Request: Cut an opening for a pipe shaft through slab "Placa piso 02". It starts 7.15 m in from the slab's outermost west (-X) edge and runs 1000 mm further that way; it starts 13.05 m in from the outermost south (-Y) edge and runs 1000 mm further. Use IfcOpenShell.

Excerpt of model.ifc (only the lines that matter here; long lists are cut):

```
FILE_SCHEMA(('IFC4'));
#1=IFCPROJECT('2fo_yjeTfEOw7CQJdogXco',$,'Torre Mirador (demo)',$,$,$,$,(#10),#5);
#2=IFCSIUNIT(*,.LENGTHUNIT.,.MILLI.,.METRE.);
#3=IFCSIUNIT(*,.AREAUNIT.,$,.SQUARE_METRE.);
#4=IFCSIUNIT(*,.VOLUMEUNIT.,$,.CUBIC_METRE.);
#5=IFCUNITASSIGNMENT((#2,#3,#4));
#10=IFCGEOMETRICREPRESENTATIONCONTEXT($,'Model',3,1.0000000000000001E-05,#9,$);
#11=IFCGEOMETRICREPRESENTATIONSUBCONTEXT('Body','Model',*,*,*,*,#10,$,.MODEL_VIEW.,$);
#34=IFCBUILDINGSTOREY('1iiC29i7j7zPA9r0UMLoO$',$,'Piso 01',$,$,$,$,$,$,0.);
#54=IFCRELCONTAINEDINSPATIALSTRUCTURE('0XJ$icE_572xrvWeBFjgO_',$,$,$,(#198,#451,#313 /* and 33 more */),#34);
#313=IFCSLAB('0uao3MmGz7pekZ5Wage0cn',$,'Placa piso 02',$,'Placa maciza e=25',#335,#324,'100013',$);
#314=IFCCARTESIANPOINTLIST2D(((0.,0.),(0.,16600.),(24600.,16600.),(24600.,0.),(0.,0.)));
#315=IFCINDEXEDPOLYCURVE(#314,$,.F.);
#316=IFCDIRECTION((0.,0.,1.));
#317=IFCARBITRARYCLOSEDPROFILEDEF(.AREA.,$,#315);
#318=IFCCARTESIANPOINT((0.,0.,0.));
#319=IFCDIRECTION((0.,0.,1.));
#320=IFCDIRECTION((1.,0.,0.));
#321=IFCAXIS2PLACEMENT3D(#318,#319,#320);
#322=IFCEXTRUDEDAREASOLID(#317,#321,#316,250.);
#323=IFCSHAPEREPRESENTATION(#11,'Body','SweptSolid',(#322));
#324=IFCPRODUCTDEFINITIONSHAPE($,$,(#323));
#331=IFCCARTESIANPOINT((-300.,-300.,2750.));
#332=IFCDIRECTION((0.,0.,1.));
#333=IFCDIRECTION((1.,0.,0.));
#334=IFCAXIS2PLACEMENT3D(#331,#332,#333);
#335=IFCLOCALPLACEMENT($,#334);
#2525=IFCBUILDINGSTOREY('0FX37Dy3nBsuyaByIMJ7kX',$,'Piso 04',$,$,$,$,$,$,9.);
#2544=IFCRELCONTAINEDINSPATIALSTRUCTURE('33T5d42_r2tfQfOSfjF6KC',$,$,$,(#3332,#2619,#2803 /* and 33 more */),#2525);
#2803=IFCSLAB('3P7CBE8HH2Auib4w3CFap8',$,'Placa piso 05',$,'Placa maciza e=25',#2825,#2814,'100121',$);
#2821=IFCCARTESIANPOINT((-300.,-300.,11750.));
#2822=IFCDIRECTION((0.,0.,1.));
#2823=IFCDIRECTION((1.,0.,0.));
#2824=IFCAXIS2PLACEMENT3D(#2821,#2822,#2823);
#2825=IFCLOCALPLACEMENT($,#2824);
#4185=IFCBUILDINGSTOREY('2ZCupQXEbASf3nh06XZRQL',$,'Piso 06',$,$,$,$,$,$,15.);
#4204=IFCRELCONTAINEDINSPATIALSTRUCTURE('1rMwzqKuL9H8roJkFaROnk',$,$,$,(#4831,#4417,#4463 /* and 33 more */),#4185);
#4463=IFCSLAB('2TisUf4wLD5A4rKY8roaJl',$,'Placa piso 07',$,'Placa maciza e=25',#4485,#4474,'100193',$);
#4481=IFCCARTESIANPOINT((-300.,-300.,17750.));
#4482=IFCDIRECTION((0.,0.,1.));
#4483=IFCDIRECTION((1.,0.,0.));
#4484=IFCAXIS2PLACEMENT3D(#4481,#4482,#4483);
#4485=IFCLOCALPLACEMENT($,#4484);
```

```python
import numpy as np
import ifcopenshell
import ifcopenshell.api.feature
import ifcopenshell.api.geometry
import ifcopenshell.api.root
import ifcopenshell.geom
import ifcopenshell.util.placement
import ifcopenshell.util.representation
import ifcopenshell.util.shape
import ifcopenshell.util.unit

model = ifcopenshell.open("model.ifc")
unit_scale = ifcopenshell.util.unit.calculate_unit_scale(model)
settings = ifcopenshell.geom.settings()


def volume(element):
    """Net volume in cubic metres, openings subtracted."""
    shape = ifcopenshell.geom.create_shape(settings, element)
    return ifcopenshell.util.shape.get_volume(shape.geometry)


slab = model.by_id(313)
before = volume(slab)

# Extent in the slab's own axes, in metres. The edges named are its -X and -Y sides.
slab_shape = ifcopenshell.geom.create_shape(settings, slab)
vertices = ifcopenshell.util.shape.get_vertices(slab_shape.geometry)
x_min, y_min, bottom = vertices.min(axis=0)
top = vertices[:, 2].max()

opening = ifcopenshell.api.root.create_entity(model, ifc_class="IfcOpeningElement", name="Pipe shaft opening", predefined_type="OPENING")
context = ifcopenshell.util.representation.get_context(model, "Model", "Body", "MODEL_VIEW")
width, depth = 1, 1
outline = [(0.0, 0.0), (width, 0.0), (width, depth), (0.0, depth), (0.0, 0.0)]
# Overshoot both faces by 50 mm so the cut is clean.
shape = ifcopenshell.api.geometry.add_slab_representation(
    model, context=context, depth=top - bottom + 0.1, polyline=outline
)
ifcopenshell.api.geometry.assign_representation(model, product=opening, representation=shape)

matrix = ifcopenshell.util.placement.get_local_placement(slab.ObjectPlacement)
matrix[:, 3] = matrix @ np.append(np.array([x_min + 7.15, y_min + 13.05, bottom - 0.05]) / unit_scale, 1.0)
ifcopenshell.api.geometry.edit_object_placement(model, product=opening, matrix=matrix, is_si=False)
ifcopenshell.api.feature.add_feature(model, feature=opening, element=slab)

after = volume(slab)

print(f"slab volume {before:.3f} -> {after:.3f} m3")

model.write("model-out.ifc")
```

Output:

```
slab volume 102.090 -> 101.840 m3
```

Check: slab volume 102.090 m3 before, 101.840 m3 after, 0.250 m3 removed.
